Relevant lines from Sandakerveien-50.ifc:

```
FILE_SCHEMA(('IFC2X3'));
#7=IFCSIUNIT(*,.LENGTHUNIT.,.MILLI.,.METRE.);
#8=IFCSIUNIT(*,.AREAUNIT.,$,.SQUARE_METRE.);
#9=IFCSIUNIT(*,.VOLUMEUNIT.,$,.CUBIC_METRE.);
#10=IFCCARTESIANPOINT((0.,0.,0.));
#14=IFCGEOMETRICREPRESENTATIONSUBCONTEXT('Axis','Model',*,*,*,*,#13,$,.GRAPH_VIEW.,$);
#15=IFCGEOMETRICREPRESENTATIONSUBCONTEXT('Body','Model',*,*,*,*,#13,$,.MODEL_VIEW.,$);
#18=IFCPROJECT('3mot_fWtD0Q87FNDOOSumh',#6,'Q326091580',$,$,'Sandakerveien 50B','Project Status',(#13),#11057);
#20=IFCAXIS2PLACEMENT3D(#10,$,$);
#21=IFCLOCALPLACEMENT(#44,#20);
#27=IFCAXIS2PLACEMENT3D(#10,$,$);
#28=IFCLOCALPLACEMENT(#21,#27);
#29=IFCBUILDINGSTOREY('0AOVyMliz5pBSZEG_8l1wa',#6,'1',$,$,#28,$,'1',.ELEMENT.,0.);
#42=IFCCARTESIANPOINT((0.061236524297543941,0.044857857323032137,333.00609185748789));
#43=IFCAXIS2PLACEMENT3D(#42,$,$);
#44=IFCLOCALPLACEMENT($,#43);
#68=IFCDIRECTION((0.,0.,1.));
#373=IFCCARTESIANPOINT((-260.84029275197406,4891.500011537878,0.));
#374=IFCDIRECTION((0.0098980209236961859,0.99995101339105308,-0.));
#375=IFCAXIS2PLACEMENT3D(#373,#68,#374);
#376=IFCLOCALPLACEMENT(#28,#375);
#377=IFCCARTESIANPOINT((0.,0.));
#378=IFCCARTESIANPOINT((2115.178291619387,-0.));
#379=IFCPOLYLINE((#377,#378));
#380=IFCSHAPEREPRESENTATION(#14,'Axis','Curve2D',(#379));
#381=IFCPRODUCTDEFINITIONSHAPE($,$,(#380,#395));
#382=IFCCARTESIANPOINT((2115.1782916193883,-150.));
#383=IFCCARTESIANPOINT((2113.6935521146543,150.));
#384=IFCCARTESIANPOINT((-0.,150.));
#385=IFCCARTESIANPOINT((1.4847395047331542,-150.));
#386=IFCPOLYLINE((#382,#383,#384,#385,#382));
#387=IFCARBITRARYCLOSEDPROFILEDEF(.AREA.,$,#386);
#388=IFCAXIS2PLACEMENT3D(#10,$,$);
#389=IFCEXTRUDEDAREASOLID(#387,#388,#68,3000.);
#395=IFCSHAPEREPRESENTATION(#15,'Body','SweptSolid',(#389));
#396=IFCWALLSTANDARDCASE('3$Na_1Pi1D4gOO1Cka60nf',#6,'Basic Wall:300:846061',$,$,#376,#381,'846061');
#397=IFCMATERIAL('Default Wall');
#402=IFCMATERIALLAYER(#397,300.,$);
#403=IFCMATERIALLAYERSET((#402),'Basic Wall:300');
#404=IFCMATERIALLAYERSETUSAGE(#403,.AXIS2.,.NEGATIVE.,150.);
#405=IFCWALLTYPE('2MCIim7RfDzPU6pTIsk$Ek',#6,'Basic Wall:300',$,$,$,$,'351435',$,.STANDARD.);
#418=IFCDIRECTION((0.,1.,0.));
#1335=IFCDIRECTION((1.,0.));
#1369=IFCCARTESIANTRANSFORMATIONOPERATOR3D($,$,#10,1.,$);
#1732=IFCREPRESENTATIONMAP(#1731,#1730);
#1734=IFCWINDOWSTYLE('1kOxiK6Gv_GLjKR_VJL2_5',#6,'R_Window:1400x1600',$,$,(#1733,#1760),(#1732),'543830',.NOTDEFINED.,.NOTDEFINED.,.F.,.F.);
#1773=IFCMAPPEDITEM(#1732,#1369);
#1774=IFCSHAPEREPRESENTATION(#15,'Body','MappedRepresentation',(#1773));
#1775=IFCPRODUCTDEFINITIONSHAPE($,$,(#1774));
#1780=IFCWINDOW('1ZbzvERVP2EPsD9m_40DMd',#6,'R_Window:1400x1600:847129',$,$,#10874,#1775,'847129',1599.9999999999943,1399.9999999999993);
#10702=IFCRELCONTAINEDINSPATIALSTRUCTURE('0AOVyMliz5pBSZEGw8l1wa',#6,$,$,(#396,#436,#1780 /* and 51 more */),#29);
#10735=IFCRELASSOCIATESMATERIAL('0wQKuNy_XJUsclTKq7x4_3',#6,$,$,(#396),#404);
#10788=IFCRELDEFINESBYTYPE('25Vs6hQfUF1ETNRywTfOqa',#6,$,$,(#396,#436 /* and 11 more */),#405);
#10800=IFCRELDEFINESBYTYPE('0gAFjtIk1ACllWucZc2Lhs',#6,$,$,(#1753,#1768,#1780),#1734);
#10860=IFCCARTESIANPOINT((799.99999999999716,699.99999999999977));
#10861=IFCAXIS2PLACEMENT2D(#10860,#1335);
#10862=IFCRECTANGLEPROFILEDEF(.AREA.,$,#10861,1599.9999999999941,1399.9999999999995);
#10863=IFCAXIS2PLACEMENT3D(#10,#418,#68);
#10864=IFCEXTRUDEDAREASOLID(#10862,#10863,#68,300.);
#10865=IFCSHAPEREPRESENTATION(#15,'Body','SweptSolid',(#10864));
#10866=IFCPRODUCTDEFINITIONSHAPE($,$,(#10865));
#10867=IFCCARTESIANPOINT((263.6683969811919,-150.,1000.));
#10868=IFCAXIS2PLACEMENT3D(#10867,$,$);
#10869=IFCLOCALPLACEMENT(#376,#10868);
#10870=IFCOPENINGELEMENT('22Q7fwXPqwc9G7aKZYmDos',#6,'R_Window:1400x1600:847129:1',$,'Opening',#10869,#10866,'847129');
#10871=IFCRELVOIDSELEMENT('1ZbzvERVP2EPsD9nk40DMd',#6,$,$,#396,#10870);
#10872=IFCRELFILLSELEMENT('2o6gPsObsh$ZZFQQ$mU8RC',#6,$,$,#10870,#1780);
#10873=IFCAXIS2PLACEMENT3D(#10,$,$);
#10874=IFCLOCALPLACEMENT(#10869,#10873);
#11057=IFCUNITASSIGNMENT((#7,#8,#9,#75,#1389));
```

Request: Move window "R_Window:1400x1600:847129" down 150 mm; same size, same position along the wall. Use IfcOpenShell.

```python
import numpy as np
import ifcopenshell
import ifcopenshell.api.geometry
import ifcopenshell.util.placement
import ifcopenshell.util.unit

model = ifcopenshell.open("Sandakerveien-50.ifc")
unit_scale = ifcopenshell.util.unit.calculate_unit_scale(model)

window = model.by_guid("1ZbzvERVP2EPsD9m_40DMd")
opening = window.FillsVoids[0].RelatingOpeningElement
dz = -150.0

shift = np.array([0.0, 0.0, dz])
# The window is placed relative to its opening, so it follows when the opening moves.
matrix = ifcopenshell.util.placement.get_local_placement(opening.ObjectPlacement)
matrix[:3, 3] += shift
ifcopenshell.api.geometry.edit_object_placement(
    model, product=opening, matrix=matrix, is_si=False, should_transform_children=True
)

print(f"moved by {dz * unit_scale:+.3f} m")

model.write("Sandakerveien-50-out.ifc")
```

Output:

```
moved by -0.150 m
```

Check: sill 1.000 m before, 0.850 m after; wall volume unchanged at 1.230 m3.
